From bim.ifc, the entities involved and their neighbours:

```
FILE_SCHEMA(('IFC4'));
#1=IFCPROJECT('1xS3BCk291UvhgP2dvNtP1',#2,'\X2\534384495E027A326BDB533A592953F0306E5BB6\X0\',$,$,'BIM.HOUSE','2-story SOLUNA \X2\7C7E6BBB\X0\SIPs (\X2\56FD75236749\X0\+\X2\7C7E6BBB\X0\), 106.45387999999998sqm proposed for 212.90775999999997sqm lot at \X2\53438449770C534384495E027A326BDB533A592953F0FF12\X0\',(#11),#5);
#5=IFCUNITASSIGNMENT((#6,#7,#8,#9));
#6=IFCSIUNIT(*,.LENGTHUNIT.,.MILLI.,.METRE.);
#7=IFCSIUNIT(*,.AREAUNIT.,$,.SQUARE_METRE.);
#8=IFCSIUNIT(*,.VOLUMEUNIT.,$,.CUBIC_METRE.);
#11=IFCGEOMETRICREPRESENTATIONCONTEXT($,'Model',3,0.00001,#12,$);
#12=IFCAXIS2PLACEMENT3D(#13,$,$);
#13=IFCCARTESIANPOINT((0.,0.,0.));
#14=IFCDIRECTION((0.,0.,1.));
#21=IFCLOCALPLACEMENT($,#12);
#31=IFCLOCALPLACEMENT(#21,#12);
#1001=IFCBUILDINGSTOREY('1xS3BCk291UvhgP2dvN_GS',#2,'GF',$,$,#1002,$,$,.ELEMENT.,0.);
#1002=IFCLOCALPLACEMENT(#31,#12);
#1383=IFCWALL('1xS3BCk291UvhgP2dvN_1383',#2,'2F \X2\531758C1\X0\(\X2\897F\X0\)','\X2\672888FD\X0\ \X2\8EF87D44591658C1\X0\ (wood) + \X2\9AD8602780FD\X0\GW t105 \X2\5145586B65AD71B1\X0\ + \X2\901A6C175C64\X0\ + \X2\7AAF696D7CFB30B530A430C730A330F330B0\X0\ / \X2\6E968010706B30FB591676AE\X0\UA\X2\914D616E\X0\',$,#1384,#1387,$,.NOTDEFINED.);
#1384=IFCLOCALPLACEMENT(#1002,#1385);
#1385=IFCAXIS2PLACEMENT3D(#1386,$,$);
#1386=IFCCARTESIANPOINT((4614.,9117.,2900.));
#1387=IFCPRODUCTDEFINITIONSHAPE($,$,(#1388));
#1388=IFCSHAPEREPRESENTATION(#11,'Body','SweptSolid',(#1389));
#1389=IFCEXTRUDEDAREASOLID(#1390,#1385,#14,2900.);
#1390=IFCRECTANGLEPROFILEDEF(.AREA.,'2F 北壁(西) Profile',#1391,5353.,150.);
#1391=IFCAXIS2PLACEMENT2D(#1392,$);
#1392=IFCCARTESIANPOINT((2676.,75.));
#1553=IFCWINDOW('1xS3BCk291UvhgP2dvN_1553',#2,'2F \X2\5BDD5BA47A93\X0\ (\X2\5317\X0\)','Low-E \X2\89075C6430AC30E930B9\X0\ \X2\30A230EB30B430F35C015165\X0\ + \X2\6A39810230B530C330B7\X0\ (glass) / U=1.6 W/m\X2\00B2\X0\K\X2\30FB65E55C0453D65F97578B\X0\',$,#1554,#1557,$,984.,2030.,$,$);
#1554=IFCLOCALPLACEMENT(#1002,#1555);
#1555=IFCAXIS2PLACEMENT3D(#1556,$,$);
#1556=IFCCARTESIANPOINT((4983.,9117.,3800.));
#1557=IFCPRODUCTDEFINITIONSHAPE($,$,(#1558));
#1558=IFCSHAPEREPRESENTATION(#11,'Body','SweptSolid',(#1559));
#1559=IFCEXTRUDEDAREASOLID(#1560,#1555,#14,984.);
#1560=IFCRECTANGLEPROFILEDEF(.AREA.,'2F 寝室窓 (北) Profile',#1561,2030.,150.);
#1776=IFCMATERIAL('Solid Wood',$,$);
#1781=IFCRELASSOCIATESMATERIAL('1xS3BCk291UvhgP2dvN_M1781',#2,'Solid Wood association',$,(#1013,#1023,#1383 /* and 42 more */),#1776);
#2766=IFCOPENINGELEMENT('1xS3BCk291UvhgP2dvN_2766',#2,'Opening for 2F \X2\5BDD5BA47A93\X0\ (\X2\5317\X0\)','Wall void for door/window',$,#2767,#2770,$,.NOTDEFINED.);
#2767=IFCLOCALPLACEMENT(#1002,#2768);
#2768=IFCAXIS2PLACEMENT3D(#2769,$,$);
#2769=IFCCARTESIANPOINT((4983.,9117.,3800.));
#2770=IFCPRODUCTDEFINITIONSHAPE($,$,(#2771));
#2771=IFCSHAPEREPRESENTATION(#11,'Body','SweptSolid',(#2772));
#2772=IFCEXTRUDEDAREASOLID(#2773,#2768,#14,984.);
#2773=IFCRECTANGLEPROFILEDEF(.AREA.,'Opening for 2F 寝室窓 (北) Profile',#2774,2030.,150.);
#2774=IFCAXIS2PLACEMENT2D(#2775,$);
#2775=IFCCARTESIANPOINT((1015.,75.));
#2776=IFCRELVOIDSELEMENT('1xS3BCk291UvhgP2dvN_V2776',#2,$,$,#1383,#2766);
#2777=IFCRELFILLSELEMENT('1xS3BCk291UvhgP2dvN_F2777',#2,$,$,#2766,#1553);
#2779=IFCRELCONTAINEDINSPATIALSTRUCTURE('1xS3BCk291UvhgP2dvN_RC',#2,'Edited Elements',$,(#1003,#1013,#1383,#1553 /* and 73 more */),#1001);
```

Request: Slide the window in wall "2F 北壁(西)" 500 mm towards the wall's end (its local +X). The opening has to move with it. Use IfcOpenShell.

```python
import ifcopenshell
import ifcopenshell.api.geometry
import ifcopenshell.util.placement
import ifcopenshell.util.unit

model = ifcopenshell.open("bim.ifc")
unit_scale = ifcopenshell.util.unit.calculate_unit_scale(model)

window = model.by_id(1553)
opening = window.FillsVoids[0].RelatingOpeningElement
wall = opening.VoidsElements[0].RelatingBuildingElement

wall_matrix = ifcopenshell.util.placement.get_local_placement(wall.ObjectPlacement)
shift = wall_matrix[:3, 0] * 0.5 / unit_scale
before = ifcopenshell.util.placement.get_local_placement(window.ObjectPlacement)[:3, 3].copy()

# The window is not placed relative to its opening, so move both.
for product in (opening, window):
    matrix = ifcopenshell.util.placement.get_local_placement(product.ObjectPlacement)
    matrix[:3, 3] += shift
    ifcopenshell.api.geometry.edit_object_placement(model, product=product, matrix=matrix, is_si=False)

after = ifcopenshell.util.placement.get_local_placement(window.ObjectPlacement)[:3, 3]
print("window moved by", (after - before).round(3) + 0.0)

model.write("bim_v2.ifc")
```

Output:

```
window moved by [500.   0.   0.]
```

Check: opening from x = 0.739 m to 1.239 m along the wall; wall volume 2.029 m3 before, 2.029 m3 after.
